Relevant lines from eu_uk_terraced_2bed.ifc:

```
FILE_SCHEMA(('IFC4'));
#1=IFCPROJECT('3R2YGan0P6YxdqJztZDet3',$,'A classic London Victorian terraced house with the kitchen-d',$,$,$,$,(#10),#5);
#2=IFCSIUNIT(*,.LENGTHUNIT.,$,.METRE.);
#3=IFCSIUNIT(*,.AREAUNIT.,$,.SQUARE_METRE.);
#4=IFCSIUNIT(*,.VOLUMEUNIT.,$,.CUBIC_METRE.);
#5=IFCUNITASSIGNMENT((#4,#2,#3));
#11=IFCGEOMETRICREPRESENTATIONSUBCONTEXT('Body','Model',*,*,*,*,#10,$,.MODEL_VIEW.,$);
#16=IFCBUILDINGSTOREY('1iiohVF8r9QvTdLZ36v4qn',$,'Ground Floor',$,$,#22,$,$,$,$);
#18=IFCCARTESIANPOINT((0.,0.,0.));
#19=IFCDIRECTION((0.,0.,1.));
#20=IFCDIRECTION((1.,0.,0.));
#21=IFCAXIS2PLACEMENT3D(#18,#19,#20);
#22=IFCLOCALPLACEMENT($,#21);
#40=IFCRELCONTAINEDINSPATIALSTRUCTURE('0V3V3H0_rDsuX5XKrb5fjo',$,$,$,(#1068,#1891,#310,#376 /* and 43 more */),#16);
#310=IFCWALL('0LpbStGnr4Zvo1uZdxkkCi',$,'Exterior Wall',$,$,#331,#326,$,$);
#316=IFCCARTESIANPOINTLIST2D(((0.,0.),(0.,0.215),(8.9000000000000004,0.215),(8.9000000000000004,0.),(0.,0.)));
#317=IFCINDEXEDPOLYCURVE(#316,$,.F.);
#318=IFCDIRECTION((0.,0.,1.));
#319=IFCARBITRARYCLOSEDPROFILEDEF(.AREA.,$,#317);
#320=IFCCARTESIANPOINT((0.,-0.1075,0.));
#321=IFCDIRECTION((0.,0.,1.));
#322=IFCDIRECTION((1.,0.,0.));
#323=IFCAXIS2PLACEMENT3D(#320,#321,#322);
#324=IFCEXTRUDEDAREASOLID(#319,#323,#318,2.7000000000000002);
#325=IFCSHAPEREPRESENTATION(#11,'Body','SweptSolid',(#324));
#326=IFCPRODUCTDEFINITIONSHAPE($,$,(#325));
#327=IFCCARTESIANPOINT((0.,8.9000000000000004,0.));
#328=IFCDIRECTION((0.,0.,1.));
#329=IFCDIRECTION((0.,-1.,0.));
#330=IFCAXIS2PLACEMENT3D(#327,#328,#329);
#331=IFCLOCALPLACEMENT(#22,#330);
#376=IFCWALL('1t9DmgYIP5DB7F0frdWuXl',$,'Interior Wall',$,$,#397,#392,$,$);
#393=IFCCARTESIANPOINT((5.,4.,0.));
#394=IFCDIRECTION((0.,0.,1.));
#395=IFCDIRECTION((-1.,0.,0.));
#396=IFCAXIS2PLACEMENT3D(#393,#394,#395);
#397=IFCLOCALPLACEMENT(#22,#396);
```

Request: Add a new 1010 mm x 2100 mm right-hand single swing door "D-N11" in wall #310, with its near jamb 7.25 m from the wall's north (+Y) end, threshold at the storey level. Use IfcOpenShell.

```python
import numpy as np
import ifcopenshell
import ifcopenshell.api.feature
import ifcopenshell.api.geometry
import ifcopenshell.api.root
import ifcopenshell.api.spatial
import ifcopenshell.geom
import ifcopenshell.util.element
import ifcopenshell.util.placement
import ifcopenshell.util.representation
import ifcopenshell.util.shape
import ifcopenshell.util.unit

model = ifcopenshell.open("eu_uk_terraced_2bed.ifc")
unit_scale = ifcopenshell.util.unit.calculate_unit_scale(model)
settings = ifcopenshell.geom.settings()


def volume(element):
    """Net volume in cubic metres, openings subtracted."""
    shape = ifcopenshell.geom.create_shape(settings, element)
    return ifcopenshell.util.shape.get_volume(shape.geometry)


wall = model.by_id(310)
storey = ifcopenshell.util.element.get_container(wall, ifc_class="IfcBuildingStorey")
context = ifcopenshell.util.representation.get_context(model, "Model", "Body", "MODEL_VIEW")
before = volume(wall)

width, height, from_end, sill = 1.01, 2.1, 7.25, 0.0  # metres

# The wall runs along its own X axis, and the end named is its -X end.
wall_shape = ifcopenshell.geom.create_shape(settings, wall)
x, y, z = ifcopenshell.util.shape.get_vertices(wall_shape.geometry).T
start = x.min() + from_end
face, thickness = float(y.min()), float(y.max() - y.min())
wall_matrix = ifcopenshell.util.placement.get_local_placement(wall.ObjectPlacement)
level = ifcopenshell.util.placement.get_local_placement(storey.ObjectPlacement)[2, 3]


def in_wall(x, y):
    """Placement at x, y metres in the wall's axes, at sill height."""
    matrix = wall_matrix.copy()
    matrix[:, 3] = wall_matrix @ np.array([x / unit_scale, y / unit_scale, 0.0, 1.0])
    matrix[2, 3] = level + sill / unit_scale
    return matrix


# Opening: a box that overshoots both wall faces by 50 mm.
opening = ifcopenshell.api.root.create_entity(model, ifc_class="IfcOpeningElement", predefined_type="OPENING")
box = ifcopenshell.api.geometry.add_wall_representation(
    model, context=context, length=width, height=height, thickness=thickness + 0.1
)
ifcopenshell.api.geometry.assign_representation(model, product=opening, representation=box)
ifcopenshell.api.geometry.edit_object_placement(model, product=opening, matrix=in_wall(start, face - 0.05), is_si=False)
ifcopenshell.api.feature.add_feature(model, feature=opening, element=wall)

door = ifcopenshell.api.root.create_entity(model, ifc_class="IfcDoor", name="D-N11", predefined_type="DOOR")
door.OverallWidth, door.OverallHeight = width / unit_scale, height / unit_scale
door.OperationType = "SINGLE_SWING_RIGHT"
body = ifcopenshell.api.geometry.add_door_representation(
    model,
    context=context,
    overall_width=door.OverallWidth,
    overall_height=door.OverallHeight,
    operation_type="SINGLE_SWING_RIGHT",
    lining_properties={"LiningDepth": thickness / unit_scale, "ThresholdDepth": thickness / unit_scale},
)
ifcopenshell.api.geometry.assign_representation(model, product=door, representation=body)
ifcopenshell.api.spatial.assign_container(model, products=[door], relating_structure=storey)
ifcopenshell.api.feature.add_filling(model, opening=opening, element=door)

# The lining spans the wall, so the door starts at the wall face.
ifcopenshell.api.geometry.edit_object_placement(model, product=door, matrix=in_wall(start, face), is_si=False)

after = volume(wall)

print(f"wall volume {before:.3f} -> {after:.3f} m3")

model.write("eu_uk_terraced_2bed_v2.ifc")
```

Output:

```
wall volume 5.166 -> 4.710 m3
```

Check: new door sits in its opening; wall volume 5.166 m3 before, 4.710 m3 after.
